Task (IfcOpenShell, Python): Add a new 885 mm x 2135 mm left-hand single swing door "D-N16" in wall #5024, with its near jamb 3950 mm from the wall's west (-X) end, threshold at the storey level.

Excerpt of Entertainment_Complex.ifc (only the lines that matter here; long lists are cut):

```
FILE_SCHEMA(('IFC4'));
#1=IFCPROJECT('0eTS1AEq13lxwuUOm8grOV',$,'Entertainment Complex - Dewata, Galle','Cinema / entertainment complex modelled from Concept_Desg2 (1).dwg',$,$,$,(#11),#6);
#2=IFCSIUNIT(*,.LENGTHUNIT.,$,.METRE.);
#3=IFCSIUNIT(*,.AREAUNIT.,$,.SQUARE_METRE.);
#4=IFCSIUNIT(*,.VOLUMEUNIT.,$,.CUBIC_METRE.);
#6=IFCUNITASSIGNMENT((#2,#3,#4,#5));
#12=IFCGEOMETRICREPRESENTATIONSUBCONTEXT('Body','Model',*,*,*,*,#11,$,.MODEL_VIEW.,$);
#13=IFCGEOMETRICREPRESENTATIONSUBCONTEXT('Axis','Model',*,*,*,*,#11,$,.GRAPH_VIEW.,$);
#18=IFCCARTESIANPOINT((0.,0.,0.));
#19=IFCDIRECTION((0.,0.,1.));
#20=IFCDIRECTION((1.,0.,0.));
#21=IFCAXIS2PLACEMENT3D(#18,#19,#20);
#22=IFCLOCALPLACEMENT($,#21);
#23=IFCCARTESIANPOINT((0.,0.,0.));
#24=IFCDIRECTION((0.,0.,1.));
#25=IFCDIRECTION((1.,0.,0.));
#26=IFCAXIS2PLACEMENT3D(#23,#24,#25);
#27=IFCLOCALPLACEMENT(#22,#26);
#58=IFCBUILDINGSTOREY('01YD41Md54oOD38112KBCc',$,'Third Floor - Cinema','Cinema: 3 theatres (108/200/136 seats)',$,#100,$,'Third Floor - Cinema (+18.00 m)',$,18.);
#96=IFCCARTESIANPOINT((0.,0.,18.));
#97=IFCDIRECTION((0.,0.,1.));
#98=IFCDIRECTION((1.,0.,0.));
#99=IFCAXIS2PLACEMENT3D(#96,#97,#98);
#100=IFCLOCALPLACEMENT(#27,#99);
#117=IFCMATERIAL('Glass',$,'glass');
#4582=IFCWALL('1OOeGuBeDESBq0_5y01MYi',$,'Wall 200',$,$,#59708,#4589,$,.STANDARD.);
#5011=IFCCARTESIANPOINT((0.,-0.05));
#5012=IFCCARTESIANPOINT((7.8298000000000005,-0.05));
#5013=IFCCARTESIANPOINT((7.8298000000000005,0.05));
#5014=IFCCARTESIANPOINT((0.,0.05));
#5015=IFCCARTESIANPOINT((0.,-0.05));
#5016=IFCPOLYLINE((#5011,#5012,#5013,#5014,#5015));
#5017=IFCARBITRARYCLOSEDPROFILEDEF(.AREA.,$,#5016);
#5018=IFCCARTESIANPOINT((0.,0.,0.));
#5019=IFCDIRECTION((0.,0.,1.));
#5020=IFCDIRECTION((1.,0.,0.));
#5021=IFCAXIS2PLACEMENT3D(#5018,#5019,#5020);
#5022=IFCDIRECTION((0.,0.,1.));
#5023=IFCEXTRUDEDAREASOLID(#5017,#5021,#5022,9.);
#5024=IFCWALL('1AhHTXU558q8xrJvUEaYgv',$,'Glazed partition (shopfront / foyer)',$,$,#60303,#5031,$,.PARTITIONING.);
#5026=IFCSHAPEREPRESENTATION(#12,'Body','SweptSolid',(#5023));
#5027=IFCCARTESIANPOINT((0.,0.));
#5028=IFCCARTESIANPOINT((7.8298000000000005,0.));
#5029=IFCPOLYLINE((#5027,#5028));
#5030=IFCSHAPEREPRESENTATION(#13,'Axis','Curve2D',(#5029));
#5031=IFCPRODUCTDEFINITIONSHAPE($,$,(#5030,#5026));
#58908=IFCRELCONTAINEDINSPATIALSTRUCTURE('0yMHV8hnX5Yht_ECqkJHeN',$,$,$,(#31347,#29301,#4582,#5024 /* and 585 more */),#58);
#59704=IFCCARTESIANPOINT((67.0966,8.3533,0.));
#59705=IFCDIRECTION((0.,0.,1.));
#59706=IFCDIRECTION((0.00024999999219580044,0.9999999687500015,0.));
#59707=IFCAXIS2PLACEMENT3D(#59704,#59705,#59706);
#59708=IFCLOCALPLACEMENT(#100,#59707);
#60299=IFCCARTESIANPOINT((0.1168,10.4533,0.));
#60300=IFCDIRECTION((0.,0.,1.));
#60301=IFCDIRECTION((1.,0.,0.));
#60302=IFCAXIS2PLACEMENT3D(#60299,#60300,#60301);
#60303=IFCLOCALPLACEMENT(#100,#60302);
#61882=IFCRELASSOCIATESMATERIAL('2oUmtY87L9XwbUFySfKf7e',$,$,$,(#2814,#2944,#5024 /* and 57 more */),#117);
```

```python
import numpy as np
import ifcopenshell
import ifcopenshell.api.feature
import ifcopenshell.api.geometry
import ifcopenshell.api.root
import ifcopenshell.api.spatial
import ifcopenshell.geom
import ifcopenshell.util.element
import ifcopenshell.util.placement
import ifcopenshell.util.representation
import ifcopenshell.util.shape
import ifcopenshell.util.unit

model = ifcopenshell.open("Entertainment_Complex.ifc")
unit_scale = ifcopenshell.util.unit.calculate_unit_scale(model)
settings = ifcopenshell.geom.settings()


def volume(element):
    """Net volume in cubic metres, openings subtracted."""
    shape = ifcopenshell.geom.create_shape(settings, element)
    return ifcopenshell.util.shape.get_volume(shape.geometry)


wall = model.by_guid("1AhHTXU558q8xrJvUEaYgv")
storey = ifcopenshell.util.element.get_container(wall, ifc_class="IfcBuildingStorey")
context = ifcopenshell.util.representation.get_context(model, "Model", "Body", "MODEL_VIEW")
before = volume(wall)

width, height, from_end, sill = 0.885, 2.135, 3.95, 0.0  # metres

# The wall runs along its own X axis, and the end named is its -X end.
wall_shape = ifcopenshell.geom.create_shape(settings, wall)
x, y, z = ifcopenshell.util.shape.get_vertices(wall_shape.geometry).T
start = x.min() + from_end
face, thickness = float(y.min()), float(y.max() - y.min())
wall_matrix = ifcopenshell.util.placement.get_local_placement(wall.ObjectPlacement)
level = ifcopenshell.util.placement.get_local_placement(storey.ObjectPlacement)[2, 3]


def in_wall(x, y):
    """Placement at x, y metres in the wall's axes, at sill height."""
    matrix = wall_matrix.copy()
    matrix[:, 3] = wall_matrix @ np.array([x / unit_scale, y / unit_scale, 0.0, 1.0])
    matrix[2, 3] = level + sill / unit_scale
    return matrix


# Opening: a box that overshoots both wall faces by 50 mm.
opening = ifcopenshell.api.root.create_entity(model, ifc_class="IfcOpeningElement", predefined_type="OPENING")
box = ifcopenshell.api.geometry.add_wall_representation(
    model, context=context, length=width, height=height, thickness=thickness + 0.1
)
ifcopenshell.api.geometry.assign_representation(model, product=opening, representation=box)
ifcopenshell.api.geometry.edit_object_placement(model, product=opening, matrix=in_wall(start, face - 0.05), is_si=False)
ifcopenshell.api.feature.add_feature(model, feature=opening, element=wall)

door = ifcopenshell.api.root.create_entity(model, ifc_class="IfcDoor", name="D-N16", predefined_type="DOOR")
door.OverallWidth, door.OverallHeight = width / unit_scale, height / unit_scale
door.OperationType = "SINGLE_SWING_LEFT"
body = ifcopenshell.api.geometry.add_door_representation(
    model,
    context=context,
    overall_width=door.OverallWidth,
    overall_height=door.OverallHeight,
    operation_type="SINGLE_SWING_LEFT",
    lining_properties={"LiningDepth": thickness / unit_scale, "ThresholdDepth": thickness / unit_scale},
)
ifcopenshell.api.geometry.assign_representation(model, product=door, representation=body)
ifcopenshell.api.spatial.assign_container(model, products=[door], relating_structure=storey)
ifcopenshell.api.feature.add_filling(model, opening=opening, element=door)

# The lining spans the wall, so the door starts at the wall face.
ifcopenshell.api.geometry.edit_object_placement(model, product=door, matrix=in_wall(start, face), is_si=False)

after = volume(wall)

print(f"wall volume {before:.3f} -> {after:.3f} m3")

model.write("Entertainment_Complex_v2.ifc")
```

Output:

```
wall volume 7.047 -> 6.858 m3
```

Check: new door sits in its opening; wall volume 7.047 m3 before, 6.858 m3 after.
